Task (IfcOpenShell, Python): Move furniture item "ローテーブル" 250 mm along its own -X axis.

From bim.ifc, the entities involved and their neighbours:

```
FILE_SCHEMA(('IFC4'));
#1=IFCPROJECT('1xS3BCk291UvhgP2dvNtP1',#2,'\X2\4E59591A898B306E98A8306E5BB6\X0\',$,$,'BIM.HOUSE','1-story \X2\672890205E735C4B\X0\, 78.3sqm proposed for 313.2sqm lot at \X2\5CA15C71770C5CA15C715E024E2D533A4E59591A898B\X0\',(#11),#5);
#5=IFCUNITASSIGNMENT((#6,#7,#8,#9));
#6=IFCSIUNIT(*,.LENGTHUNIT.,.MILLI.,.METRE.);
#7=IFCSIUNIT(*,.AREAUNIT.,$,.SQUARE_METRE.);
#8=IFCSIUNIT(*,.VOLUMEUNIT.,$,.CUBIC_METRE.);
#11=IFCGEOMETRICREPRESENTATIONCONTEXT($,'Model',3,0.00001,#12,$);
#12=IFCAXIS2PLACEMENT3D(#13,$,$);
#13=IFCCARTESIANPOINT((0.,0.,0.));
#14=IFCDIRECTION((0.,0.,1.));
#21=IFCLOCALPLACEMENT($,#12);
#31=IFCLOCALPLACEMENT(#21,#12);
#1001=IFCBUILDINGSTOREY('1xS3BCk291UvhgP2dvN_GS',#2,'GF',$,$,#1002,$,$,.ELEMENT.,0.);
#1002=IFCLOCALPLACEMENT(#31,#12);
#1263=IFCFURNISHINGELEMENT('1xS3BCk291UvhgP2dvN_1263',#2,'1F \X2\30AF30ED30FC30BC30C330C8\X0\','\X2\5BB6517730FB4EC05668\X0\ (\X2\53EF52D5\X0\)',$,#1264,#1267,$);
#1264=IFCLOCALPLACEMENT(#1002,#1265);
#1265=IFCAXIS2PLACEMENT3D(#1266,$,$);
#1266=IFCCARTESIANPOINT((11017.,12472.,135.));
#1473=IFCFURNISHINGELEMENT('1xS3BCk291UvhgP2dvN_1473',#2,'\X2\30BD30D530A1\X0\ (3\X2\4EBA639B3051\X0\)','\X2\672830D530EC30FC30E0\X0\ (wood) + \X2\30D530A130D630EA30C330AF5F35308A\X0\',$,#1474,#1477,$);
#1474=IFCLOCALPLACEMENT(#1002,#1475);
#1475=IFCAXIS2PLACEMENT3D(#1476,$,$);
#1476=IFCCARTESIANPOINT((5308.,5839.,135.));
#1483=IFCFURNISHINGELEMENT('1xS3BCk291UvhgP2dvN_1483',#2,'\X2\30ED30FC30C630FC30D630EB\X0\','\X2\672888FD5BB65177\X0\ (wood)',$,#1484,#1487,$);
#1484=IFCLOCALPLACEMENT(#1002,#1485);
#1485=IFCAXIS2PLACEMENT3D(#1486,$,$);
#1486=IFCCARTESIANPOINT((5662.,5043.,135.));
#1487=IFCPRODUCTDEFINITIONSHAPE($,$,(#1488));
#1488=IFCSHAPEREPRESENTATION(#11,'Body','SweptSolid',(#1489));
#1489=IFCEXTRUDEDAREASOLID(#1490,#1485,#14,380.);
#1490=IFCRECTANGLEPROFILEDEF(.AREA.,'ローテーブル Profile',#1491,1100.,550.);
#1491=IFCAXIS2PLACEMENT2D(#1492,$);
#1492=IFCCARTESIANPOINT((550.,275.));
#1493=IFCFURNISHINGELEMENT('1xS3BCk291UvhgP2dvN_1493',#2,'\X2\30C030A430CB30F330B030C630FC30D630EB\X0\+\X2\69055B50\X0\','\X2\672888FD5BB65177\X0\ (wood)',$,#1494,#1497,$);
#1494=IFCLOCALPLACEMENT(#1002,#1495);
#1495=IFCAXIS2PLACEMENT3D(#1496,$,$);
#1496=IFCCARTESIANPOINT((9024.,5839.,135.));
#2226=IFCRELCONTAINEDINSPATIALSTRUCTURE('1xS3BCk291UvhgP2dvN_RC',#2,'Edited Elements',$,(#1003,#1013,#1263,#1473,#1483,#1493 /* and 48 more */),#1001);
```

```python
import ifcopenshell
import ifcopenshell.api.geometry
import ifcopenshell.util.placement

model = ifcopenshell.open("bim.ifc")

item = model.by_id(1483)
matrix = ifcopenshell.util.placement.get_local_placement(item.ObjectPlacement)
matrix[:3, 3] -= matrix[:3, 0] * 250.0
ifcopenshell.api.geometry.edit_object_placement(model, product=item, matrix=matrix, is_si=False)

print(ifcopenshell.util.placement.get_local_placement(item.ObjectPlacement).round(3) + 0.0)

model.write("bim_updated.ifc")
```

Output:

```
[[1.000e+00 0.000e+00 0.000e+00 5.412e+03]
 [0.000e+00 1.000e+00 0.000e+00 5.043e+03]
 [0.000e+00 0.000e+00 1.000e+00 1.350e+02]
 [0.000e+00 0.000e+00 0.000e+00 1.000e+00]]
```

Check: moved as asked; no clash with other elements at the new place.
